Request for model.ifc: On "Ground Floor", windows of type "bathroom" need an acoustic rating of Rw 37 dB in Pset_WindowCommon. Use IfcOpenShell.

First a look at what the model holds.

```python
import ifcopenshell
import ifcopenshell.util.element

model = ifcopenshell.open("model.ifc")
print(model.schema)
storey = next(s for s in model.by_type("IfcBuildingStorey") if s.Name == "Ground Floor")
windows = [e for e in ifcopenshell.util.element.get_decomposition(storey) if e.is_a("IfcWindow")]
seen = {}
for e in windows:
    element_type = ifcopenshell.util.element.get_type(e)
    key = (element_type.Name if element_type != e and element_type else None, ifcopenshell.util.element.get_pset(e, "Pset_WindowCommon", "AcousticRating"))
    seen[key] = seen.get(key, 0) + 1
for (name, value), count in sorted(seen.items(), key=str):
    print(count, "x", name, "|", value)
```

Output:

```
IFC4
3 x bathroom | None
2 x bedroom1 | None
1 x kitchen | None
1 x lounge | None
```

```python
import ifcopenshell
import ifcopenshell.api.pset
import ifcopenshell.util.element

model = ifcopenshell.open("model.ifc")

storey = next(s for s in model.by_type("IfcBuildingStorey") if s.Name == "Ground Floor")
windows = [e for e in ifcopenshell.util.element.get_decomposition(storey) if e.is_a("IfcWindow")]

count = 0
for e in windows:
    element_type = ifcopenshell.util.element.get_type(e)
    if element_type in (None, e) or element_type.Name != "bathroom":
        continue
    # add_pset returns the element's existing set when there is one.
    pset = ifcopenshell.api.pset.add_pset(model, product=e, name="Pset_WindowCommon")
    ifcopenshell.api.pset.edit_pset(model, pset=pset, properties={"AcousticRating": "Rw 37 dB"})
    count += 1

print(count, "windows updated")

model.write("model_v2.ifc")
```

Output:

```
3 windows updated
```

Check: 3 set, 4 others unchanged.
